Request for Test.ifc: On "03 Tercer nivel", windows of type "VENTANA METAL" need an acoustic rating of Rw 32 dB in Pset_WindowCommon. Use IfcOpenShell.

First a look at what the model holds.

```python
import ifcopenshell
import ifcopenshell.util.element

model = ifcopenshell.open("Test.ifc")
print(model.schema)
storey = next(s for s in model.by_type("IfcBuildingStorey") if s.Name == "03 Tercer nivel")
windows = [e for e in ifcopenshell.util.element.get_decomposition(storey) if e.is_a("IfcWindow")]
seen = {}
for e in windows:
    element_type = ifcopenshell.util.element.get_type(e)
    key = (element_type.Name if element_type != e and element_type else None, ifcopenshell.util.element.get_pset(e, "Pset_WindowCommon", "AcousticRating"))
    seen[key] = seen.get(key, 0) + 1
for (name, value), count in sorted(seen.items(), key=str):
    print(count, "x", name, "|", value)
```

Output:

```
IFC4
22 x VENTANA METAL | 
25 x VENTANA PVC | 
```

```python
import ifcopenshell
import ifcopenshell.api.pset
import ifcopenshell.util.element

model = ifcopenshell.open("Test.ifc")

storey = next(s for s in model.by_type("IfcBuildingStorey") if s.Name == "03 Tercer nivel")
windows = [e for e in ifcopenshell.util.element.get_decomposition(storey) if e.is_a("IfcWindow")]

count = 0
for e in windows:
    element_type = ifcopenshell.util.element.get_type(e)
    if element_type in (None, e) or element_type.Name != "VENTANA METAL":
        continue
    # add_pset returns the element's existing set when there is one.
    pset = ifcopenshell.api.pset.add_pset(model, product=e, name="Pset_WindowCommon")
    ifcopenshell.api.pset.edit_pset(model, pset=pset, properties={"AcousticRating": "Rw 32 dB"})
    count += 1

print(count, "windows updated")

model.write("Test_v2.ifc")
```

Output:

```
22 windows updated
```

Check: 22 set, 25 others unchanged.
